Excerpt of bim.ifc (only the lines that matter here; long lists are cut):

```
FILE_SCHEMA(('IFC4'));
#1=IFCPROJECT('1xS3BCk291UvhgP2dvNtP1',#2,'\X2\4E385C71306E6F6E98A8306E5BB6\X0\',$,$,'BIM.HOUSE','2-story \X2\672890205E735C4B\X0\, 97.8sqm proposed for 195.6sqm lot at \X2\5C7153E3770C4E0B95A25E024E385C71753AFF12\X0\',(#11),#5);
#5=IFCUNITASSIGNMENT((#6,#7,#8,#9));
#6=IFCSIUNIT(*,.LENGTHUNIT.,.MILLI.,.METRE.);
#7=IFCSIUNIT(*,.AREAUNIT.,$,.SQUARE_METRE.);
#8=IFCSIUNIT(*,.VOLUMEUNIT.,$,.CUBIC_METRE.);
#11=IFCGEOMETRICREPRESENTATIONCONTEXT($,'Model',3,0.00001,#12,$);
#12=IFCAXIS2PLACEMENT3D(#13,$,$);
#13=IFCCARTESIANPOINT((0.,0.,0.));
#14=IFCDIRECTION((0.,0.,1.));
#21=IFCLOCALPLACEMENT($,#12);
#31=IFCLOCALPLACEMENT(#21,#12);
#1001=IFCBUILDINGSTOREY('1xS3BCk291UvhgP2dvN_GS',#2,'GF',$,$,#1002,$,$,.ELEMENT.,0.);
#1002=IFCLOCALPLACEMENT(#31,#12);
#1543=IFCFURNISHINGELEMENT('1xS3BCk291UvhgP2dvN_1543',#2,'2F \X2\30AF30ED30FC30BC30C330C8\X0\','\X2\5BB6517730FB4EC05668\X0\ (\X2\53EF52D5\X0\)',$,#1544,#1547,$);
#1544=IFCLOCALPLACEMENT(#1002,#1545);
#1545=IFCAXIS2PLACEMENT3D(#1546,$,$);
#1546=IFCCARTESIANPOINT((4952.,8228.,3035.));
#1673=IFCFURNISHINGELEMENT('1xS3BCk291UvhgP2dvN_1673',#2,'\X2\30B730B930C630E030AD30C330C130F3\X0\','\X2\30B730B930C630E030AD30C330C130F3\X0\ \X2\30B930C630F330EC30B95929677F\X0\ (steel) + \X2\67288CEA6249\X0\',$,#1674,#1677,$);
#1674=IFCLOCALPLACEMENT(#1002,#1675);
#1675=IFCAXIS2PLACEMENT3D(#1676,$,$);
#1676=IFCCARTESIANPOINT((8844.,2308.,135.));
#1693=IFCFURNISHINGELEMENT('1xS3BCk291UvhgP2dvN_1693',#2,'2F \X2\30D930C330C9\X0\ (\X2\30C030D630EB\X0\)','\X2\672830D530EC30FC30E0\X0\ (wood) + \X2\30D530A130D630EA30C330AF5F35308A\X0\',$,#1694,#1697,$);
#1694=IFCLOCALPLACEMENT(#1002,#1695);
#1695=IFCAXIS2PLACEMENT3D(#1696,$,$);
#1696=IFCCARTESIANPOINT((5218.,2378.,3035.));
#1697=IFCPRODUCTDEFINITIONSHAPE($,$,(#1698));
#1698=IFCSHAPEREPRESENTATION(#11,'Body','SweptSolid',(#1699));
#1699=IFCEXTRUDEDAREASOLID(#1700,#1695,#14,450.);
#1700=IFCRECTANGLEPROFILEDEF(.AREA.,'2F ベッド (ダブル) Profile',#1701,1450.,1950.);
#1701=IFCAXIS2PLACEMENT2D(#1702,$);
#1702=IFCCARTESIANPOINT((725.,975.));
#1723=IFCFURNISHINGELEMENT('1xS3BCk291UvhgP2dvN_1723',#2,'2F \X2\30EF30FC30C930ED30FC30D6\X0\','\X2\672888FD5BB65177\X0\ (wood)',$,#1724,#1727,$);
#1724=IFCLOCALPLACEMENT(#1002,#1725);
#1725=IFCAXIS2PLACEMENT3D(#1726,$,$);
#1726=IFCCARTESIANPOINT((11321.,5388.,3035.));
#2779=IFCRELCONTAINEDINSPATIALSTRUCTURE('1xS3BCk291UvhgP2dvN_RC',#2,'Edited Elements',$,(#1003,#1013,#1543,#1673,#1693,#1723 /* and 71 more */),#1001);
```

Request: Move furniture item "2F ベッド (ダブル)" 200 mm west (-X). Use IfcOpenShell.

```python
import ifcopenshell
import ifcopenshell.api.geometry
import ifcopenshell.util.placement
import ifcopenshell.util.unit

model = ifcopenshell.open("bim.ifc")
unit_scale = ifcopenshell.util.unit.calculate_unit_scale(model)

item = model.by_guid("1xS3BCk291UvhgP2dvN_1693")
matrix = ifcopenshell.util.placement.get_local_placement(item.ObjectPlacement)
matrix[0, 3] -= 0.2 / unit_scale
ifcopenshell.api.geometry.edit_object_placement(model, product=item, matrix=matrix, is_si=False)

print(ifcopenshell.util.placement.get_local_placement(item.ObjectPlacement).round(3) + 0.0)

model.write("bim_v2.ifc")
```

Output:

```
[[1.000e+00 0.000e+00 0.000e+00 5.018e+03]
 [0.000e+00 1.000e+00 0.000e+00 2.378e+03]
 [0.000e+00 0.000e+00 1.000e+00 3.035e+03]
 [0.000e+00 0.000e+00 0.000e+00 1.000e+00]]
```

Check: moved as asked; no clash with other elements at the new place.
